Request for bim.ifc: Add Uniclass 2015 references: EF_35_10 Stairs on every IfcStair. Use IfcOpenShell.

First a look at what the model holds.

```python
import ifcopenshell

model = ifcopenshell.open("bim.ifc")
print(model.schema)
print("classifications:", [c.Name for c in model.by_type("IfcClassification")])
for ifc_class in ("IfcDoor", "IfcRoof", "IfcStair", "IfcWall", "IfcWindow"):
    print(ifc_class, len(model.by_type(ifc_class)))
```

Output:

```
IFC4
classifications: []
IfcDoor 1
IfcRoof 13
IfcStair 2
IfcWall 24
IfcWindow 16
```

```python
import ifcopenshell
import ifcopenshell.api.classification

model = ifcopenshell.open("bim.ifc")

system = ifcopenshell.api.classification.add_classification(model, classification="Uniclass 2015")

codes = {
    "IfcStair": ("EF_35_10", "Stairs"),
}
for ifc_class, (code, name) in codes.items():
    products = model.by_type(ifc_class)
    ifcopenshell.api.classification.add_reference(
        model, products=products, classification=system, identification=code, name=name
    )
    print(code, len(products))

model.write("bim-out.ifc")
```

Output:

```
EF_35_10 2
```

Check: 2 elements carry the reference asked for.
